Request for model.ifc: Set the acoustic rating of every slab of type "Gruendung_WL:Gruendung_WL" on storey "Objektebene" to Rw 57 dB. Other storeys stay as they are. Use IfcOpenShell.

First a look at what the model holds.

```python
import ifcopenshell
import ifcopenshell.util.element

model = ifcopenshell.open("model.ifc")
print(model.schema)
storey = next(s for s in model.by_type("IfcBuildingStorey") if s.Name == "Objektebene")
slabs = [e for e in ifcopenshell.util.element.get_decomposition(storey) if e.is_a("IfcSlab")]
seen = {}
for e in slabs:
    element_type = ifcopenshell.util.element.get_type(e)
    key = (element_type.Name if element_type != e and element_type else None, ifcopenshell.util.element.get_pset(e, "Pset_SlabCommon", "AcousticRating"))
    seen[key] = seen.get(key, 0) + 1
for (name, value), count in sorted(seen.items(), key=str):
    print(count, "x", name, "|", value)
```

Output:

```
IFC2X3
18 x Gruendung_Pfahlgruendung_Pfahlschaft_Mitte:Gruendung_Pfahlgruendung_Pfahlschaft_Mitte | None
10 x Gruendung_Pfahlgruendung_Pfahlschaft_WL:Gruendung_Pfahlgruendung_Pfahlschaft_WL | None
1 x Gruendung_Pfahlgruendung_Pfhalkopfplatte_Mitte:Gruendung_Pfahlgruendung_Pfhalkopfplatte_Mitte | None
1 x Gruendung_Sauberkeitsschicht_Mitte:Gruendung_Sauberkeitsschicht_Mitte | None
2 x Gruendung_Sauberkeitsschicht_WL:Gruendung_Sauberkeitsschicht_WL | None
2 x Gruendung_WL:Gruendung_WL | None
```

```python
import ifcopenshell
import ifcopenshell.api.pset
import ifcopenshell.util.element

model = ifcopenshell.open("model.ifc")

storey = next(s for s in model.by_type("IfcBuildingStorey") if s.Name == "Objektebene")
slabs = [e for e in ifcopenshell.util.element.get_decomposition(storey) if e.is_a("IfcSlab")]

count = 0
for e in slabs:
    element_type = ifcopenshell.util.element.get_type(e)
    if element_type in (None, e) or element_type.Name != "Gruendung_WL:Gruendung_WL":
        continue
    # add_pset returns the element's existing set when there is one.
    pset = ifcopenshell.api.pset.add_pset(model, product=e, name="Pset_SlabCommon")
    ifcopenshell.api.pset.edit_pset(model, pset=pset, properties={"AcousticRating": "Rw 57 dB"})
    count += 1

print(count, "slabs updated")

model.write("model_edited.ifc")
```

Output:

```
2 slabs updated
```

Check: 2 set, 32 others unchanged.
